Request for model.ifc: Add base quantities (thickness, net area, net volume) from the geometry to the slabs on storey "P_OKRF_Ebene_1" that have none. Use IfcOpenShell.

First a look at what the model holds.

```python
import ifcopenshell
import ifcopenshell.util.element
import ifcopenshell.util.unit

model = ifcopenshell.open("model.ifc")
print(model.schema)
for unit_type in ("LENGTHUNIT", "AREAUNIT", "VOLUMEUNIT"):
    print(unit_type, ifcopenshell.util.unit.calculate_unit_scale(model, unit_type))
storey = next(s for s in model.by_type("IfcBuildingStorey") if s.Name == "P_OKRF_Ebene_1")
slabs = [e for e in ifcopenshell.util.element.get_decomposition(storey) if e.is_a("IfcSlab")]
for e in sorted(slabs, key=lambda e: e.id()):
    print(e.id(), e.is_a(), e.Name, list(ifcopenshell.util.element.get_psets(e, qtos_only=True)), sep=" | ")
```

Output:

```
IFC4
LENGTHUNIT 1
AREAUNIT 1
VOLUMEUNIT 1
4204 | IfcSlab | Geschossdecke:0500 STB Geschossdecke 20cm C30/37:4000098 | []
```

```python
import ifcopenshell
import ifcopenshell.api.pset
import ifcopenshell.geom
import ifcopenshell.util.element
import ifcopenshell.util.shape
import ifcopenshell.util.unit

model = ifcopenshell.open("model.ifc")
unit_scale = ifcopenshell.util.unit.calculate_unit_scale(model)
area_scale = ifcopenshell.util.unit.calculate_unit_scale(model, "AREAUNIT")
volume_scale = ifcopenshell.util.unit.calculate_unit_scale(model, "VOLUMEUNIT")
settings = ifcopenshell.geom.settings()

storey = next(s for s in model.by_type("IfcBuildingStorey") if s.Name == "P_OKRF_Ebene_1")
slabs = [e for e in ifcopenshell.util.element.get_decomposition(storey) if e.is_a("IfcSlab")]

for e in sorted(slabs, key=lambda e: e.id()):
    if ifcopenshell.util.element.get_psets(e, qtos_only=True, should_inherit=False):
        continue
    # Geometry comes back in metres, in the element's own axes.
    shape = ifcopenshell.geom.create_shape(settings, e)
    values = {
        "Width": ifcopenshell.util.shape.get_z(shape.geometry) / unit_scale,
        "NetArea": ifcopenshell.util.shape.get_footprint_area(shape.geometry) / area_scale,
        "NetVolume": ifcopenshell.util.shape.get_volume(shape.geometry) / volume_scale,
    }
    qto = ifcopenshell.api.pset.add_qto(model, product=e, name="Qto_SlabBaseQuantities")
    ifcopenshell.api.pset.edit_qto(model, qto=qto, properties=values)
    print(e.id(), {k: round(v, 3) for k, v in values.items()})

model.write("model_v2.ifc")
```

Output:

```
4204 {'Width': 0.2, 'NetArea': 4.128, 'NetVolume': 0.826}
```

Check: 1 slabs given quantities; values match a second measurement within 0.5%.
